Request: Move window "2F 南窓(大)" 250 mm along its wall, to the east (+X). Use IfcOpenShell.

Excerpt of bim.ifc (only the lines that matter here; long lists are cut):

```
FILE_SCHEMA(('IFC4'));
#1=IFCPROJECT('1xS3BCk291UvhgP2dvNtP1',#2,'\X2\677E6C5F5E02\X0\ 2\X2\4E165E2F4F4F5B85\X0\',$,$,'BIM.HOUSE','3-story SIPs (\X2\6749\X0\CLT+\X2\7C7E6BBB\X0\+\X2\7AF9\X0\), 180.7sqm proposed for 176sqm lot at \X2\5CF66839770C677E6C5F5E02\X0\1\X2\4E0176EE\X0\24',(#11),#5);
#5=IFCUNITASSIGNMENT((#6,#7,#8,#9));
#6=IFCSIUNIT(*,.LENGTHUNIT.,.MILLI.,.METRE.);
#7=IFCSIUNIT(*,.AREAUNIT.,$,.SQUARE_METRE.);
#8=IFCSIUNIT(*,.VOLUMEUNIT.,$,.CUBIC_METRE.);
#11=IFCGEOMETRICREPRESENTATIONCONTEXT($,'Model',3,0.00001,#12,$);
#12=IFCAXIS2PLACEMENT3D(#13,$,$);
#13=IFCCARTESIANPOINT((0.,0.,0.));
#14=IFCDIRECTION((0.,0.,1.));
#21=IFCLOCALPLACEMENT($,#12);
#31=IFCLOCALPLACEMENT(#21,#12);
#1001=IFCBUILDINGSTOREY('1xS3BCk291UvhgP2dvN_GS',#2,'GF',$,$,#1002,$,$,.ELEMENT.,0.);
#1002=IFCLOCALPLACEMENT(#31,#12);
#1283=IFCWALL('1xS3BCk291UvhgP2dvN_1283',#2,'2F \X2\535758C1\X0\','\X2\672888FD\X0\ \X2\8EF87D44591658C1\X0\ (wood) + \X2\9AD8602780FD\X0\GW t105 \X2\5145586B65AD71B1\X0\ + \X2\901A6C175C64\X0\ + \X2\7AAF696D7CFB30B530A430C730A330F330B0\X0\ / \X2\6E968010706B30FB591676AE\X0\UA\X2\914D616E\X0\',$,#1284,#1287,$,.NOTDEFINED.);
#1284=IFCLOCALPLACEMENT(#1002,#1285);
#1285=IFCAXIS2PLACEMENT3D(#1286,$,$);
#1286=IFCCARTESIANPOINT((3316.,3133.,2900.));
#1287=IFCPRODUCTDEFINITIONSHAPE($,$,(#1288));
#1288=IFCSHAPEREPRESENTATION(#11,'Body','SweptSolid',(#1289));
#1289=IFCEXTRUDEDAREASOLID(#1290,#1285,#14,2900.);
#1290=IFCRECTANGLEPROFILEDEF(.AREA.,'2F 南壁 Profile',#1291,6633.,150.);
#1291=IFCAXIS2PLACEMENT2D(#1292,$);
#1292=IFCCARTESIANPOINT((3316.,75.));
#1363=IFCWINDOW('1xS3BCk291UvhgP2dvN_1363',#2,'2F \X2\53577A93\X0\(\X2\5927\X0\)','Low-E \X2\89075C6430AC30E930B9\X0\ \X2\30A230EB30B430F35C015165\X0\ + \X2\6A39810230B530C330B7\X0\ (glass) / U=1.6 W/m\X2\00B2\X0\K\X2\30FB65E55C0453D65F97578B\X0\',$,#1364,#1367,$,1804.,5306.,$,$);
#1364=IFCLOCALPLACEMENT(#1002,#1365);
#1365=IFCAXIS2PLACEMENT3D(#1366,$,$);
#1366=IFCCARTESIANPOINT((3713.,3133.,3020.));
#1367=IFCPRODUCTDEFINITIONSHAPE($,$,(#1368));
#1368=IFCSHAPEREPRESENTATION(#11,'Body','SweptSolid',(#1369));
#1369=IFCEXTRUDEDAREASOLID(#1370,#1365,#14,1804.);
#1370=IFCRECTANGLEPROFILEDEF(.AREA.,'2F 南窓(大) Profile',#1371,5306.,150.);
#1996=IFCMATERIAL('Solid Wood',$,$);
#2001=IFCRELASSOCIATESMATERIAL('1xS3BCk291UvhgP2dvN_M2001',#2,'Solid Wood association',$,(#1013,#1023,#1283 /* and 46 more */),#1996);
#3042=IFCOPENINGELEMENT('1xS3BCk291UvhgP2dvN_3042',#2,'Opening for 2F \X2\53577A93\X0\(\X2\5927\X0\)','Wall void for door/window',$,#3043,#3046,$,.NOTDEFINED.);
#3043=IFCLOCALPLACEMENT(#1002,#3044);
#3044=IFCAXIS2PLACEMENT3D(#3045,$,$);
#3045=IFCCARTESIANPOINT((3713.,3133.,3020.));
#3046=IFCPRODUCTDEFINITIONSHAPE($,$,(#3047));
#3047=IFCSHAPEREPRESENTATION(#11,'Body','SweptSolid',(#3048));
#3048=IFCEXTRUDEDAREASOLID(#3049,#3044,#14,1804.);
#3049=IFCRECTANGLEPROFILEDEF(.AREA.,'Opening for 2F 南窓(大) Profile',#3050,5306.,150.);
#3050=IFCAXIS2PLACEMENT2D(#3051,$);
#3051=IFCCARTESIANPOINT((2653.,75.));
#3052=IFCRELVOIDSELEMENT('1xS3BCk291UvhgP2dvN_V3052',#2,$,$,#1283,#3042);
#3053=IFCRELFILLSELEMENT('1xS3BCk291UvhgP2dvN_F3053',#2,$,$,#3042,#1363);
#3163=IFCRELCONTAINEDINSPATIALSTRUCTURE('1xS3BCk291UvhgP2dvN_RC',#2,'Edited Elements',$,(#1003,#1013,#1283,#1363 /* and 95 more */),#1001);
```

```python
import ifcopenshell
import ifcopenshell.api.geometry
import ifcopenshell.util.placement

model = ifcopenshell.open("bim.ifc")

window = model.by_id(1363)
opening = window.FillsVoids[0].RelatingOpeningElement
wall = opening.VoidsElements[0].RelatingBuildingElement

wall_matrix = ifcopenshell.util.placement.get_local_placement(wall.ObjectPlacement)
shift = wall_matrix[:3, 0] * 250.0
before = ifcopenshell.util.placement.get_local_placement(window.ObjectPlacement)[:3, 3].copy()

# The window is not placed relative to its opening, so move both.
for product in (opening, window):
    matrix = ifcopenshell.util.placement.get_local_placement(product.ObjectPlacement)
    matrix[:3, 3] += shift
    ifcopenshell.api.geometry.edit_object_placement(model, product=product, matrix=matrix, is_si=False)

after = ifcopenshell.util.placement.get_local_placement(window.ObjectPlacement)[:3, 3]
print("window moved by", (after - before).round(3) + 0.0)

model.write("bim_rev.ifc")
```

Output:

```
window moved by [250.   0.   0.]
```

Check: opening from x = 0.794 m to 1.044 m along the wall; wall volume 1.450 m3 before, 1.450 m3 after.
